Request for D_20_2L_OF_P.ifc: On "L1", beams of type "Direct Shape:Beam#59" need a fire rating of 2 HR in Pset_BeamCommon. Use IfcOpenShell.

First a look at what the model holds.

```python
import ifcopenshell
import ifcopenshell.util.element

model = ifcopenshell.open("D_20_2L_OF_P.ifc")
print(model.schema)
storey = next(s for s in model.by_type("IfcBuildingStorey") if s.Name == "L1")
beams = [e for e in ifcopenshell.util.element.get_decomposition(storey) if e.is_a("IfcBeam")]
seen = {}
for e in beams:
    element_type = ifcopenshell.util.element.get_type(e)
    key = (element_type.Name if element_type != e and element_type else None, ifcopenshell.util.element.get_pset(e, "Pset_BeamCommon", "FireRating"))
    seen[key] = seen.get(key, 0) + 1
for (name, value), count in sorted(seen.items(), key=str):
    print(count, "x", name, "|", value)
```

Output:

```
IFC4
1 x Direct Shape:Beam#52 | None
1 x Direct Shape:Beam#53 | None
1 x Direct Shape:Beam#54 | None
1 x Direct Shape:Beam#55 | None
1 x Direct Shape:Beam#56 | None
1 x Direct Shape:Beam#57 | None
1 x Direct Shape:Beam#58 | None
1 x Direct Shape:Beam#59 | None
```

```python
import ifcopenshell
import ifcopenshell.api.pset
import ifcopenshell.util.element

model = ifcopenshell.open("D_20_2L_OF_P.ifc")

storey = next(s for s in model.by_type("IfcBuildingStorey") if s.Name == "L1")
beams = [e for e in ifcopenshell.util.element.get_decomposition(storey) if e.is_a("IfcBeam")]

count = 0
for e in beams:
    element_type = ifcopenshell.util.element.get_type(e)
    if element_type in (None, e) or element_type.Name != "Direct Shape:Beam#59":
        continue
    # add_pset returns the element's existing set when there is one.
    pset = ifcopenshell.api.pset.add_pset(model, product=e, name="Pset_BeamCommon")
    ifcopenshell.api.pset.edit_pset(model, pset=pset, properties={"FireRating": "2 HR"})
    count += 1

print(count, "beams updated")

model.write("D_20_2L_OF_P_edited.ifc")
```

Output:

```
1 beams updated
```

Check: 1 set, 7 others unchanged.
